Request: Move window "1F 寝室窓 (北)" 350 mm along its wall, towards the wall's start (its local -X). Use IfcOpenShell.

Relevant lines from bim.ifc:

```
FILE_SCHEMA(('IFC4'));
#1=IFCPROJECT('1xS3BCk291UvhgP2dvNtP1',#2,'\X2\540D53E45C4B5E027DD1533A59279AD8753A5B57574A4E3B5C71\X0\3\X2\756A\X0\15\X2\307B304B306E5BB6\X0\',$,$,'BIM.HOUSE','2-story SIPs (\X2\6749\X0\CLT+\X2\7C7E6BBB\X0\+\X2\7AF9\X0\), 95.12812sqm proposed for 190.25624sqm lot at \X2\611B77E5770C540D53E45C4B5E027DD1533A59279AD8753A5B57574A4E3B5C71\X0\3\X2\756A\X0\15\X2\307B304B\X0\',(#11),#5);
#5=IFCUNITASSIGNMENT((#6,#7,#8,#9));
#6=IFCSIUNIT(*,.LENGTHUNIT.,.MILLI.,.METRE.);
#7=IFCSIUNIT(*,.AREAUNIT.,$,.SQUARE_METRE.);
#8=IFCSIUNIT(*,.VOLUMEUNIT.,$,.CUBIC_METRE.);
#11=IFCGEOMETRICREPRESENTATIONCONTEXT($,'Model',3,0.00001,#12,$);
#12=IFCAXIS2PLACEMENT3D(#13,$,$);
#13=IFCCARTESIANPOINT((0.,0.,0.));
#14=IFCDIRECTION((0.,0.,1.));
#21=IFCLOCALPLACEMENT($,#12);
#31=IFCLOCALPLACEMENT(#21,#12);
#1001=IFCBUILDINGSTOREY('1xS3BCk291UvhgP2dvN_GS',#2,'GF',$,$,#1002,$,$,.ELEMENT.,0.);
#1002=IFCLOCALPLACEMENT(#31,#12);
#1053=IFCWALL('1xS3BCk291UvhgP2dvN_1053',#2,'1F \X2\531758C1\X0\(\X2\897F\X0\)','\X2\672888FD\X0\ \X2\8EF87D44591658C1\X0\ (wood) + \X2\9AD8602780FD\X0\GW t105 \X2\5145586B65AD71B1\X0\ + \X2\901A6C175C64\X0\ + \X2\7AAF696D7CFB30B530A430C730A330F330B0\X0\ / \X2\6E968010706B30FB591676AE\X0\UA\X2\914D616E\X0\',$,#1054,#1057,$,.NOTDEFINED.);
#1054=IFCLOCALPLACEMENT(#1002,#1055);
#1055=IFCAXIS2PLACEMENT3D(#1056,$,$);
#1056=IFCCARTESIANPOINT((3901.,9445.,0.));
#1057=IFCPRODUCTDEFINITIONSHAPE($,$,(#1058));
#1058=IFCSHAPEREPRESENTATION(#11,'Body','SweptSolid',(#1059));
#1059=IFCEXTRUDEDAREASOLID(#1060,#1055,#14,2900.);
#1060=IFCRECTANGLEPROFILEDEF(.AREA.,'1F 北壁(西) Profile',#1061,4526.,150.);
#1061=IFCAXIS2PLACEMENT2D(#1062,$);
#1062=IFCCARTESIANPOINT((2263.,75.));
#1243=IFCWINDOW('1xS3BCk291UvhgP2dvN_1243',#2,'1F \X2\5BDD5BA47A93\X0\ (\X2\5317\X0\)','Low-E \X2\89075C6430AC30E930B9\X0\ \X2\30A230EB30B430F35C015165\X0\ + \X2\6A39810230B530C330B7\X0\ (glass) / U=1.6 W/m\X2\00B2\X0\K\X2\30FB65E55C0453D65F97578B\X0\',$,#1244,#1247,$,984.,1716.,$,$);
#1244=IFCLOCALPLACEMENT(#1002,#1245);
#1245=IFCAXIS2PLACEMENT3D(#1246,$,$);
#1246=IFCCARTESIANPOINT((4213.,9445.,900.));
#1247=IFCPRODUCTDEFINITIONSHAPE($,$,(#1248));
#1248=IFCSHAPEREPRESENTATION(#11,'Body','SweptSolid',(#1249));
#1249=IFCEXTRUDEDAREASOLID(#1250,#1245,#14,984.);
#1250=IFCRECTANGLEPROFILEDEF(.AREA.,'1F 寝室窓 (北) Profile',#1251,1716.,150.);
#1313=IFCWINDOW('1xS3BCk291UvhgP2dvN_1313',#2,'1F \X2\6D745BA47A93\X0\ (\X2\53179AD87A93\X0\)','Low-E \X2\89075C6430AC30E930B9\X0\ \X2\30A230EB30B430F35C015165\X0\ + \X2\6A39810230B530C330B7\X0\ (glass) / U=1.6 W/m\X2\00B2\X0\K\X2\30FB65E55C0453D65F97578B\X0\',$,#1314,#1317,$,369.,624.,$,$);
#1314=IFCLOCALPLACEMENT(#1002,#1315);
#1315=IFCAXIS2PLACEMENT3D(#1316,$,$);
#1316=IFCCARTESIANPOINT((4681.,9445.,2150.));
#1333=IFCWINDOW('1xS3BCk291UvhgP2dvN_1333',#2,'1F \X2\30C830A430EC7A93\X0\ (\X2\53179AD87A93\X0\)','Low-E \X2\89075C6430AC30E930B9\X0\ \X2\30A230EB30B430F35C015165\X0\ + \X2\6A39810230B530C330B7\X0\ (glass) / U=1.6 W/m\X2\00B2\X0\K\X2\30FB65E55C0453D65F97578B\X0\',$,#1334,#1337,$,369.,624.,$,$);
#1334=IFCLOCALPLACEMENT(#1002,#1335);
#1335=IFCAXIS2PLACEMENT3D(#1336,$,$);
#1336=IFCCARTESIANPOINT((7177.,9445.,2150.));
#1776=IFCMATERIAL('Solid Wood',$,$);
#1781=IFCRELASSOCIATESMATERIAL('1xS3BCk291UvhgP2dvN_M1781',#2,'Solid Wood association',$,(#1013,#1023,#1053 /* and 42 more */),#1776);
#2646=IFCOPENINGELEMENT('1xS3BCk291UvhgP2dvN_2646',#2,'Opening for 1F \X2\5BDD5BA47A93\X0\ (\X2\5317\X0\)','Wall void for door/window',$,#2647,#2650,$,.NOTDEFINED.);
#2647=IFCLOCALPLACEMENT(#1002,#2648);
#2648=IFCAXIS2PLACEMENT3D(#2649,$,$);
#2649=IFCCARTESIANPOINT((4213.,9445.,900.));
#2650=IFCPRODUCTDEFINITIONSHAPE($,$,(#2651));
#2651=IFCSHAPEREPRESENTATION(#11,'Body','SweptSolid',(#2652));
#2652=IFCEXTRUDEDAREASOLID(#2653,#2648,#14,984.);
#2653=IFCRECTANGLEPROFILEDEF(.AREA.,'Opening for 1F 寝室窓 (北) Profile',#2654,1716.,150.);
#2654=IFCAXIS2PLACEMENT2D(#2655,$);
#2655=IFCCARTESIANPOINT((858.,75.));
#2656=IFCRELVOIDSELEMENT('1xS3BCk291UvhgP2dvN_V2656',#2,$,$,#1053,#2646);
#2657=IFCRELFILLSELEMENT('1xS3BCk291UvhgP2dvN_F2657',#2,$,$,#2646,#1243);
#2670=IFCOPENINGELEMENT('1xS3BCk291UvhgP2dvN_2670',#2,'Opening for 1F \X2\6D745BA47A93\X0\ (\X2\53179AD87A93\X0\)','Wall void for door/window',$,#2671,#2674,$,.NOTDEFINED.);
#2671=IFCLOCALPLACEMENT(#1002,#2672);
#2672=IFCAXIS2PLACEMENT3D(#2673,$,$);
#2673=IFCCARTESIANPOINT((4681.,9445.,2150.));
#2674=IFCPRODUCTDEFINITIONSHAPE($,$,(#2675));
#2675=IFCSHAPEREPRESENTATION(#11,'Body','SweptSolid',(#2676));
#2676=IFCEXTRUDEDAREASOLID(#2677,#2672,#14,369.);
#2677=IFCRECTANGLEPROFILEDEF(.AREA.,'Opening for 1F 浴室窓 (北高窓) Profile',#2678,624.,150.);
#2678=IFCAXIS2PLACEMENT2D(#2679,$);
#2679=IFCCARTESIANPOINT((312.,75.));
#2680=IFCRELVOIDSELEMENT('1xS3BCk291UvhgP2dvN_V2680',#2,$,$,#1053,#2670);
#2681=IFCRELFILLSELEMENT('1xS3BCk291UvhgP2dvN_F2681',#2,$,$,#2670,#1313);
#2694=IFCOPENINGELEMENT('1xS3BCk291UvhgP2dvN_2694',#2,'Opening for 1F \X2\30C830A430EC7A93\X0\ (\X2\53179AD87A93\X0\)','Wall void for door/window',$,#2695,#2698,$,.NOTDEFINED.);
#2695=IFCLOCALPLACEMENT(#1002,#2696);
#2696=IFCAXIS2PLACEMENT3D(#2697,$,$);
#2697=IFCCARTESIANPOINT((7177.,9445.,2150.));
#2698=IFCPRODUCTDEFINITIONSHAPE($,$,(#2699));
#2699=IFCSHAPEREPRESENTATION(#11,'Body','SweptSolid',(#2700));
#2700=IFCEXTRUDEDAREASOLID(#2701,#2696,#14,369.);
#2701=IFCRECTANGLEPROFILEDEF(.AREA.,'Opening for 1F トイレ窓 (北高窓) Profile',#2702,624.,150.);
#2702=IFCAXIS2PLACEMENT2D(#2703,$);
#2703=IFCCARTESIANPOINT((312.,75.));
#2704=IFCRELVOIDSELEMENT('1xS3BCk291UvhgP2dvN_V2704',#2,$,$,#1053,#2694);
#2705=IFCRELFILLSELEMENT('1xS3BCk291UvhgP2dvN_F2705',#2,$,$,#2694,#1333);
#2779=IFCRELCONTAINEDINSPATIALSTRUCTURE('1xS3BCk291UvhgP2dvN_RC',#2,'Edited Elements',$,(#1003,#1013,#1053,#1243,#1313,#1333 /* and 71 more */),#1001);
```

```python
import ifcopenshell
import ifcopenshell.api.geometry
import ifcopenshell.util.placement
import ifcopenshell.util.unit

model = ifcopenshell.open("bim.ifc")
unit_scale = ifcopenshell.util.unit.calculate_unit_scale(model)

window = model.by_guid("1xS3BCk291UvhgP2dvN_1243")
opening = window.FillsVoids[0].RelatingOpeningElement
wall = opening.VoidsElements[0].RelatingBuildingElement

wall_matrix = ifcopenshell.util.placement.get_local_placement(wall.ObjectPlacement)
shift = wall_matrix[:3, 0] * -0.35 / unit_scale
before = ifcopenshell.util.placement.get_local_placement(window.ObjectPlacement)[:3, 3].copy()

# The window is not placed relative to its opening, so move both.
for product in (opening, window):
    matrix = ifcopenshell.util.placement.get_local_placement(product.ObjectPlacement)
    matrix[:3, 3] += shift
    ifcopenshell.api.geometry.edit_object_placement(model, product=product, matrix=matrix, is_si=False)

after = ifcopenshell.util.placement.get_local_placement(window.ObjectPlacement)[:3, 3]
print("window moved by", (after - before).round(3) + 0.0)

model.write("bim_updated.ifc")
```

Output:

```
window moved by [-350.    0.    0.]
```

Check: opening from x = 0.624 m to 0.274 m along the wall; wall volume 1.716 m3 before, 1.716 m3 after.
